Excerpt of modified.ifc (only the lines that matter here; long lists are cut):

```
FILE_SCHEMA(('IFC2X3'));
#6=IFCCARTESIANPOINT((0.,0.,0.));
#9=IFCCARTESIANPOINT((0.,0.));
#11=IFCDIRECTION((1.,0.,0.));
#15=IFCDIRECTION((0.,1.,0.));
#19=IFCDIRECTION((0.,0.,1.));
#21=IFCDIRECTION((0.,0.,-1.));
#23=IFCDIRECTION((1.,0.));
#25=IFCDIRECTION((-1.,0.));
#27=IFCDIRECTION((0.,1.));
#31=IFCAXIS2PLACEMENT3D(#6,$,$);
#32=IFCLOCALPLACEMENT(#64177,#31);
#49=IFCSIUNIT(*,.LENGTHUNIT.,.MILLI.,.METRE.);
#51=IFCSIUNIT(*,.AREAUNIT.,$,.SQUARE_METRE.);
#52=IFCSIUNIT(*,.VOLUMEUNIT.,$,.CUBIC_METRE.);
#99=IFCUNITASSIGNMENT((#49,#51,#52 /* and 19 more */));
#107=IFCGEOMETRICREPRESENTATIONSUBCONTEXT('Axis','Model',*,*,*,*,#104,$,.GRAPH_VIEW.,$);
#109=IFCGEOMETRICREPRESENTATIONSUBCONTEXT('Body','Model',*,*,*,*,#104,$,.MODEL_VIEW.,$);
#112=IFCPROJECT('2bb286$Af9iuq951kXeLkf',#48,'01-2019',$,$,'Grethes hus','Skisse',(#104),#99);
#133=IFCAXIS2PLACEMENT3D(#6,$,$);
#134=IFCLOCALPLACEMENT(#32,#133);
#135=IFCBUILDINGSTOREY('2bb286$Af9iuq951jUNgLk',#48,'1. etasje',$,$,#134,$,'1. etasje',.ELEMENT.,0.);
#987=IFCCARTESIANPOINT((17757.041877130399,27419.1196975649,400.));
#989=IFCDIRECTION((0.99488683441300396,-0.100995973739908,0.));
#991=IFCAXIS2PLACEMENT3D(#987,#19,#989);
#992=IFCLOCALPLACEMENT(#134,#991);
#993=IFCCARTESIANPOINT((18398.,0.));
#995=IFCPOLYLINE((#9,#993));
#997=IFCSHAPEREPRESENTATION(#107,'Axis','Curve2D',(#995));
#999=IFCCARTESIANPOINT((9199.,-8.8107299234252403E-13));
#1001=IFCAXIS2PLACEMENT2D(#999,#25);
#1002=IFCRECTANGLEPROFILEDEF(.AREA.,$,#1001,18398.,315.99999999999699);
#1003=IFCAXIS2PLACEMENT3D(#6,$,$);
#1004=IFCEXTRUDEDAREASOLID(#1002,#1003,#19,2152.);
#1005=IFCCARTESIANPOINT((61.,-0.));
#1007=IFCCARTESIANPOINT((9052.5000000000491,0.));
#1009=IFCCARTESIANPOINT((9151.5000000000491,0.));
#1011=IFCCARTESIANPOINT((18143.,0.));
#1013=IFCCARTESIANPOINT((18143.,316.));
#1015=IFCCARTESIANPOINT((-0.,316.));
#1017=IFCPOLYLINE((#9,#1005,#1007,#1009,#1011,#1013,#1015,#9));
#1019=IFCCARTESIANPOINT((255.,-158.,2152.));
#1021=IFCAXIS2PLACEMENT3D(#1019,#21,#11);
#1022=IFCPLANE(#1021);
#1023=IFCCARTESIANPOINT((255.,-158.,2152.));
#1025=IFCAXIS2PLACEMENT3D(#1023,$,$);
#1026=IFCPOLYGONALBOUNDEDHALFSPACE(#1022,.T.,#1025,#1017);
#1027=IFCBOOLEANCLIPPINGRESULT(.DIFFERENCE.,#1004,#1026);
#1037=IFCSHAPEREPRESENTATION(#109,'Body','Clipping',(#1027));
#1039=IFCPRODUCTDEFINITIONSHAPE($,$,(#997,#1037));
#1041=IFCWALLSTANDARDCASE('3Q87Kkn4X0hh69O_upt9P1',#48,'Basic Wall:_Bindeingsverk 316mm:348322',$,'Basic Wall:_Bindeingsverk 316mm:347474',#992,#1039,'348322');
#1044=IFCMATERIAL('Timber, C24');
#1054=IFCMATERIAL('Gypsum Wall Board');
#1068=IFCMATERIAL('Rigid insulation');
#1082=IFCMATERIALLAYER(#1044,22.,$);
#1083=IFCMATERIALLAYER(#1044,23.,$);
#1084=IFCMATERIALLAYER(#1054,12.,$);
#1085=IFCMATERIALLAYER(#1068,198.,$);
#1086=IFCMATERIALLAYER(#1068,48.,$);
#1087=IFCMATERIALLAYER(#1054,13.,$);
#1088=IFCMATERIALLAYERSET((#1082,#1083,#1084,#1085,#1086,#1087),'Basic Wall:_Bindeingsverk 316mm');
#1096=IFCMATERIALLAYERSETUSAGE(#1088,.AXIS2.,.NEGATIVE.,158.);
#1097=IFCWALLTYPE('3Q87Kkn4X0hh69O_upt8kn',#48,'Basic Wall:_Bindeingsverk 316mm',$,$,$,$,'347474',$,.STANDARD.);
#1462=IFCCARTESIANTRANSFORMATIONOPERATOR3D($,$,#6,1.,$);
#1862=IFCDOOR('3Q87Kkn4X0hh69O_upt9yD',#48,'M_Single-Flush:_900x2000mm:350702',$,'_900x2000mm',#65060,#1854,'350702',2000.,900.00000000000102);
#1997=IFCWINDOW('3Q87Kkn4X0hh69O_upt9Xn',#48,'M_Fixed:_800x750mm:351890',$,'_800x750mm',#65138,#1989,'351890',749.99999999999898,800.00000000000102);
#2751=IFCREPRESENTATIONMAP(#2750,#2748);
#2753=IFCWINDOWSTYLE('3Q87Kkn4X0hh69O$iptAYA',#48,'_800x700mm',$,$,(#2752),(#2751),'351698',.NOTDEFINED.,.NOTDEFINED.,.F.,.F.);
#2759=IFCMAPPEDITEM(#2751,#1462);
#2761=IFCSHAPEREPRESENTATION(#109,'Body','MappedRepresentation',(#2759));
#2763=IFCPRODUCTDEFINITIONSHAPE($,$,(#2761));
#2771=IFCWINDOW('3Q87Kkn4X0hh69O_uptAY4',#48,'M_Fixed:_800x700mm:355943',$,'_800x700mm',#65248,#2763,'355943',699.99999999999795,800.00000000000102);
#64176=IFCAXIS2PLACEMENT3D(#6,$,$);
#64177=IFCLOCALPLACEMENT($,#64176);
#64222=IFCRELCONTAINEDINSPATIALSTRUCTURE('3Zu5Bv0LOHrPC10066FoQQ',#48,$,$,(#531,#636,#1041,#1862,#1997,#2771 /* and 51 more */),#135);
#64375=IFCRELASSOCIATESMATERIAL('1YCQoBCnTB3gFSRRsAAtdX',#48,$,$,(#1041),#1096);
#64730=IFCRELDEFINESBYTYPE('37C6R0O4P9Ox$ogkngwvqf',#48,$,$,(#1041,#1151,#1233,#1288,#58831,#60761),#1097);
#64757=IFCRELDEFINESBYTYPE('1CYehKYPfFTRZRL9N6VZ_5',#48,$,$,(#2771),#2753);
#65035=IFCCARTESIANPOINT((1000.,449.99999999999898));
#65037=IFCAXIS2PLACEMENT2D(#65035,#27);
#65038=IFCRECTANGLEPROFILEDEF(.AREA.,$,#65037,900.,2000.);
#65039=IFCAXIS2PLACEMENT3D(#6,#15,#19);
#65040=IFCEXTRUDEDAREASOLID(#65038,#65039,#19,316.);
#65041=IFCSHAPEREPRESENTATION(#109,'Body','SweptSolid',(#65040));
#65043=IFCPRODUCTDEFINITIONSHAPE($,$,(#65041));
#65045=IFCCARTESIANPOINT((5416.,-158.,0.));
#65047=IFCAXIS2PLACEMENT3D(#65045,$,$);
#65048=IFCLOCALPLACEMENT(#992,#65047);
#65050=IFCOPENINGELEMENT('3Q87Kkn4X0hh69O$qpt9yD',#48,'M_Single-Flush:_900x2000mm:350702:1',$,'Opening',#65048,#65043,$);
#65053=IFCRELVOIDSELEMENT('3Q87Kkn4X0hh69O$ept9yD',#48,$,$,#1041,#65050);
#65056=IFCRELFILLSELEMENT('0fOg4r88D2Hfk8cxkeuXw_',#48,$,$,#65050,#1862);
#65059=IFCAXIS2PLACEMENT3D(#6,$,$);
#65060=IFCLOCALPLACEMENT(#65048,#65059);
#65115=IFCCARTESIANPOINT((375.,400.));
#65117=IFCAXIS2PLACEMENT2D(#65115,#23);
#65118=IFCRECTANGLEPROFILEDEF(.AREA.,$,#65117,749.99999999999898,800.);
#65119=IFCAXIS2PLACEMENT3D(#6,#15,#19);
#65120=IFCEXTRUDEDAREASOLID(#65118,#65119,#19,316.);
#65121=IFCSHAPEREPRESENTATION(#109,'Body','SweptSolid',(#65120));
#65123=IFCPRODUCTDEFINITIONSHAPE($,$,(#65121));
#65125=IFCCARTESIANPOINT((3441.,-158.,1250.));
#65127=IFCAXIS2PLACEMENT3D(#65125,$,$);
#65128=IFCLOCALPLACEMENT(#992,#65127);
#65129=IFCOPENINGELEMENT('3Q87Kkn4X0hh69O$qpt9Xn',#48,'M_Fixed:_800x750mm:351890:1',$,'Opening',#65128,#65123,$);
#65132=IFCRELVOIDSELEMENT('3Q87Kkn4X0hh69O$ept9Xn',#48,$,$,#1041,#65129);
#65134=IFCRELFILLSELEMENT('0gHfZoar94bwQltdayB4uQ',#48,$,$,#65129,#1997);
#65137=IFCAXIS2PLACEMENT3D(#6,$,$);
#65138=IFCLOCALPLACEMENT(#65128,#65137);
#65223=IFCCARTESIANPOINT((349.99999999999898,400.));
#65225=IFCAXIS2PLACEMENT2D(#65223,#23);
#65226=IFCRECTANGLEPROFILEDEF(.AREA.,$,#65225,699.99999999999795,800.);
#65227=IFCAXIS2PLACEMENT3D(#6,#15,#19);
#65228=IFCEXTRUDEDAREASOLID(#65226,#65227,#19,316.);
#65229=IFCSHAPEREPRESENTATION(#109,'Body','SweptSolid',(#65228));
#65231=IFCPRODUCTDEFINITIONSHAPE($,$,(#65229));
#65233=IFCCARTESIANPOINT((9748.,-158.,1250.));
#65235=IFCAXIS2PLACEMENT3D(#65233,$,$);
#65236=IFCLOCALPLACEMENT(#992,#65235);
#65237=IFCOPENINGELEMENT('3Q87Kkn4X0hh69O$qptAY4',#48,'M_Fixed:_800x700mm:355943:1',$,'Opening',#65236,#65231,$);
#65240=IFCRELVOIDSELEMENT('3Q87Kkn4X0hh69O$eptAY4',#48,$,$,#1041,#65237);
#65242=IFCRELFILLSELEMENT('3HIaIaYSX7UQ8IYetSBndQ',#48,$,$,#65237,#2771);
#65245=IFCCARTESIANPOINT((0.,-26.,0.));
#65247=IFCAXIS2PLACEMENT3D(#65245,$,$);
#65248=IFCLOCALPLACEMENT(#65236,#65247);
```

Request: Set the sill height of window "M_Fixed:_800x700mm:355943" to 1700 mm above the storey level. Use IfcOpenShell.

```python
import numpy as np
import ifcopenshell
import ifcopenshell.api.geometry
import ifcopenshell.geom
import ifcopenshell.util.element
import ifcopenshell.util.placement
import ifcopenshell.util.shape
import ifcopenshell.util.unit

model = ifcopenshell.open("modified.ifc")
unit_scale = ifcopenshell.util.unit.calculate_unit_scale(model)

window = model.by_guid("3Q87Kkn4X0hh69O_uptAY4")
opening = window.FillsVoids[0].RelatingOpeningElement
storey = ifcopenshell.util.element.get_container(window, ifc_class="IfcBuildingStorey")
level = ifcopenshell.util.placement.get_local_placement(storey.ObjectPlacement)[2, 3]

# The opening's origin need not be at the sill, so measure its lowest point.
shape = ifcopenshell.geom.create_shape(ifcopenshell.geom.settings(), opening)
bottom = ifcopenshell.util.shape.get_shape_bottom_elevation(shape, shape.geometry) / unit_scale
dz = level + 1.7 / unit_scale - bottom

shift = np.array([0.0, 0.0, dz])
# The window is placed relative to its opening, so it follows when the opening moves.
matrix = ifcopenshell.util.placement.get_local_placement(opening.ObjectPlacement)
matrix[:3, 3] += shift
ifcopenshell.api.geometry.edit_object_placement(
    model, product=opening, matrix=matrix, is_si=False, should_transform_children=True
)

print(f"moved by {dz * unit_scale:+.3f} m")

model.write("modified_v2.ifc")
```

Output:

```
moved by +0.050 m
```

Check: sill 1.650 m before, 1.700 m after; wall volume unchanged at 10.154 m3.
